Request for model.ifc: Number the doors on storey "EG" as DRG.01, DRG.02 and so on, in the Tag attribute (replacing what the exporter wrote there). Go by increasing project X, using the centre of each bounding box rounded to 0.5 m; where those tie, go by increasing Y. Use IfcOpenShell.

First a look at what the model holds.

```python
import ifcopenshell
import ifcopenshell.util.element
import ifcopenshell.util.placement

model = ifcopenshell.open("model.ifc")
print(model.schema)
storey = next(s for s in model.by_type("IfcBuildingStorey") if s.Name == "EG")
doors = [e for e in ifcopenshell.util.element.get_decomposition(storey) if e.is_a("IfcDoor")]
for e in sorted(doors, key=lambda e: e.id()):
    origin = ifcopenshell.util.placement.get_local_placement(e.ObjectPlacement)[:3, 3]
    print(e.id(), e.Tag, e.Name, origin.round(2) + 0.0, sep=" | ")
```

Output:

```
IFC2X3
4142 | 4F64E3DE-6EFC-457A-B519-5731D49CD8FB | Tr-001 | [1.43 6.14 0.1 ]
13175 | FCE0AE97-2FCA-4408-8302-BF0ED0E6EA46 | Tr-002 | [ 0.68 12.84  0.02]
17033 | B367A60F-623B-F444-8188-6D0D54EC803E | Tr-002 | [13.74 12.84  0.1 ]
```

```python
import ifcopenshell
import ifcopenshell.geom
import ifcopenshell.util.element
import ifcopenshell.util.shape

model = ifcopenshell.open("model.ifc")
settings = ifcopenshell.geom.settings()
settings.set("use-world-coords", True)


def centre(element):
    shape = ifcopenshell.geom.create_shape(settings, element)
    return ifcopenshell.util.shape.get_bbox_centroid(shape.geometry)


storey = next(s for s in model.by_type("IfcBuildingStorey") if s.Name == "EG")
doors = [e for e in ifcopenshell.util.element.get_decomposition(storey) if e.is_a("IfcDoor")]

# Insertion points can sit at a corner or the storey origin, so sort by the geometry (in metres).
centres = {e: centre(e) for e in doors}
doors.sort(key=lambda e: (round(centres[e][0] / 0.5), centres[e][1]))

for i, e in enumerate(doors, start=1):
    number = f"DRG.{i:02d}"
    e.Tag = number
    print(e.id(), number)

model.write("model_v2.ifc")
```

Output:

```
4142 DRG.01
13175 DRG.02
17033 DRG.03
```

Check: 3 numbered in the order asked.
